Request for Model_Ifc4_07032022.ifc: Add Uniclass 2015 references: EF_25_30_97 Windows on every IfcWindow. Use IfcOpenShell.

First a look at what the model holds.

```python
import ifcopenshell

model = ifcopenshell.open("Model_Ifc4_07032022.ifc")
print(model.schema)
print("classifications:", [c.Name for c in model.by_type("IfcClassification")])
for ifc_class in ("IfcDoor", "IfcRoof", "IfcStair", "IfcWall", "IfcWindow"):
    print(ifc_class, len(model.by_type(ifc_class)))
```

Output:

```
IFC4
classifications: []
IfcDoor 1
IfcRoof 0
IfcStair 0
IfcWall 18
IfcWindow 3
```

```python
import ifcopenshell
import ifcopenshell.api.classification

model = ifcopenshell.open("Model_Ifc4_07032022.ifc")

system = ifcopenshell.api.classification.add_classification(model, classification="Uniclass 2015")

codes = {
    "IfcWindow": ("EF_25_30_97", "Windows"),
}
for ifc_class, (code, name) in codes.items():
    products = model.by_type(ifc_class)
    ifcopenshell.api.classification.add_reference(
        model, products=products, classification=system, identification=code, name=name
    )
    print(code, len(products))

model.write("Model_Ifc4_07032022_updated.ifc")
```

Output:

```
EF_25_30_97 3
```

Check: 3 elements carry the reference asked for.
